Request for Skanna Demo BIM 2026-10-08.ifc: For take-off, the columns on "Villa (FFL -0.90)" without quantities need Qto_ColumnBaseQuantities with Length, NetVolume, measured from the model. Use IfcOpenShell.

First a look at what the model holds.

```python
import ifcopenshell
import ifcopenshell.util.element
import ifcopenshell.util.unit

model = ifcopenshell.open("Skanna Demo BIM 2026-10-08.ifc")
print(model.schema)
for unit_type in ("LENGTHUNIT", "AREAUNIT", "VOLUMEUNIT"):
    print(unit_type, ifcopenshell.util.unit.calculate_unit_scale(model, unit_type))
storey = next(s for s in model.by_type("IfcBuildingStorey") if s.Name == "Villa (FFL -0.90)")
columns = [e for e in ifcopenshell.util.element.get_decomposition(storey) if e.is_a("IfcColumn")]
for e in sorted(columns, key=lambda e: e.id()):
    print(e.id(), e.is_a(), e.Name, list(ifcopenshell.util.element.get_psets(e, qtos_only=True)), sep=" | ")
```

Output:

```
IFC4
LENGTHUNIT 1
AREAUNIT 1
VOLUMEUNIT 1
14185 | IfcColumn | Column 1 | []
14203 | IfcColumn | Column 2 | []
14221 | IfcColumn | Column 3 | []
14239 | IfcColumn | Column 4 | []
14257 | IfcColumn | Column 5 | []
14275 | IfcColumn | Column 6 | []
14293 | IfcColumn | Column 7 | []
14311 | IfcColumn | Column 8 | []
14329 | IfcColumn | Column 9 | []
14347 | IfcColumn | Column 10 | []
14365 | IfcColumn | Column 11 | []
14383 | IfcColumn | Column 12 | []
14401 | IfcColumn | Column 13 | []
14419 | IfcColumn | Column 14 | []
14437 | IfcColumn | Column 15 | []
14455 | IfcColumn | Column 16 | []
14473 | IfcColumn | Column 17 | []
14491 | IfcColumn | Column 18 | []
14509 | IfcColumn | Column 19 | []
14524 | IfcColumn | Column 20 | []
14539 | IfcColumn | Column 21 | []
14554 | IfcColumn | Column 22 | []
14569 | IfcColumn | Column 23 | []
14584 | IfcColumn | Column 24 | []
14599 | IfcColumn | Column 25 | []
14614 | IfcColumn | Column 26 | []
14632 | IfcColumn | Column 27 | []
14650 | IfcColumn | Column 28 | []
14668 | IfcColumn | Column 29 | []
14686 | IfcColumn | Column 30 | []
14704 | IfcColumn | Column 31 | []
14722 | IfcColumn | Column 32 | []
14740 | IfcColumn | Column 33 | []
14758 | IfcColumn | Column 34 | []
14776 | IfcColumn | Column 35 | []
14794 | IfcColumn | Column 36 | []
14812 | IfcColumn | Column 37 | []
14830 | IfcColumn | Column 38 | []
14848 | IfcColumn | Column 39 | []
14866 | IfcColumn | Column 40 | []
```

```python
import ifcopenshell
import ifcopenshell.api.pset
import ifcopenshell.geom
import ifcopenshell.util.element
import ifcopenshell.util.shape
import ifcopenshell.util.unit

model = ifcopenshell.open("Skanna Demo BIM 2026-10-08.ifc")
unit_scale = ifcopenshell.util.unit.calculate_unit_scale(model)
volume_scale = ifcopenshell.util.unit.calculate_unit_scale(model, "VOLUMEUNIT")
settings = ifcopenshell.geom.settings()

storey = next(s for s in model.by_type("IfcBuildingStorey") if s.Name == "Villa (FFL -0.90)")
columns = [e for e in ifcopenshell.util.element.get_decomposition(storey) if e.is_a("IfcColumn")]

for e in sorted(columns, key=lambda e: e.id()):
    if ifcopenshell.util.element.get_psets(e, qtos_only=True, should_inherit=False):
        continue
    # Geometry comes back in metres, in the element's own axes.
    shape = ifcopenshell.geom.create_shape(settings, e)
    values = {
        "Length": ifcopenshell.util.shape.get_z(shape.geometry) / unit_scale,
        "NetVolume": ifcopenshell.util.shape.get_volume(shape.geometry) / volume_scale,
    }
    qto = ifcopenshell.api.pset.add_qto(model, product=e, name="Qto_ColumnBaseQuantities")
    ifcopenshell.api.pset.edit_qto(model, qto=qto, properties=values)
    print(e.id(), {k: round(v, 3) for k, v in values.items()})

model.write("Skanna Demo BIM 2026-10-08-out.ifc")
```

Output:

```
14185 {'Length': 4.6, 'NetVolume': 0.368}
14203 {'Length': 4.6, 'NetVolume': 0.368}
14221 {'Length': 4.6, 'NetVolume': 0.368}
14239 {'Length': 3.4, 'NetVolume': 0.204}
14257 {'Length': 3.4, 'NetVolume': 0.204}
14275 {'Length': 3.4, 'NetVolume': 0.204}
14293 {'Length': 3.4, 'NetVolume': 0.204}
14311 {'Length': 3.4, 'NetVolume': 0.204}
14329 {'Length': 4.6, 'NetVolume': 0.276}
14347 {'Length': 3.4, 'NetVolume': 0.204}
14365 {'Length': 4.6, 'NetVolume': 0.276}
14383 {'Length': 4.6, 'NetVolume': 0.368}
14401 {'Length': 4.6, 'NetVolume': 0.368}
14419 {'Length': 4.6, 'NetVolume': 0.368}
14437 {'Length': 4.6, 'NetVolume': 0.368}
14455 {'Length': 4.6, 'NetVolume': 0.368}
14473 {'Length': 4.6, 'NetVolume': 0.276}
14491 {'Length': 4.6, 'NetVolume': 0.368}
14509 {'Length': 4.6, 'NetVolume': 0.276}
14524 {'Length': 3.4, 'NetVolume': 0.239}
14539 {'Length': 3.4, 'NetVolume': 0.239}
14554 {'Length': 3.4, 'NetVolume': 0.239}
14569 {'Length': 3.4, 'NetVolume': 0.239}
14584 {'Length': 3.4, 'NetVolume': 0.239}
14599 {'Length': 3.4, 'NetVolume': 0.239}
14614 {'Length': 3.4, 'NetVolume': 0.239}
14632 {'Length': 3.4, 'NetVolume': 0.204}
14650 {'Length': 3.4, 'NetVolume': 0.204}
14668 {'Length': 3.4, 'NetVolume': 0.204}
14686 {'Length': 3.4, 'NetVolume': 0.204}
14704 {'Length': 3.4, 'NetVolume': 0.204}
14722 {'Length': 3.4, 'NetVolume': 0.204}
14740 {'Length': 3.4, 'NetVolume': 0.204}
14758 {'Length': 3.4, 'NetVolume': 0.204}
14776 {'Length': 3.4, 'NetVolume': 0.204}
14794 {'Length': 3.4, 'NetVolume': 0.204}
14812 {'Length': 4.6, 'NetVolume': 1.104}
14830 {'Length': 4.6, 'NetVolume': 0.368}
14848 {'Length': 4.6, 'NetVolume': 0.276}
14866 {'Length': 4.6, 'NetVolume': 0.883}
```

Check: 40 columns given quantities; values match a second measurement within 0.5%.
